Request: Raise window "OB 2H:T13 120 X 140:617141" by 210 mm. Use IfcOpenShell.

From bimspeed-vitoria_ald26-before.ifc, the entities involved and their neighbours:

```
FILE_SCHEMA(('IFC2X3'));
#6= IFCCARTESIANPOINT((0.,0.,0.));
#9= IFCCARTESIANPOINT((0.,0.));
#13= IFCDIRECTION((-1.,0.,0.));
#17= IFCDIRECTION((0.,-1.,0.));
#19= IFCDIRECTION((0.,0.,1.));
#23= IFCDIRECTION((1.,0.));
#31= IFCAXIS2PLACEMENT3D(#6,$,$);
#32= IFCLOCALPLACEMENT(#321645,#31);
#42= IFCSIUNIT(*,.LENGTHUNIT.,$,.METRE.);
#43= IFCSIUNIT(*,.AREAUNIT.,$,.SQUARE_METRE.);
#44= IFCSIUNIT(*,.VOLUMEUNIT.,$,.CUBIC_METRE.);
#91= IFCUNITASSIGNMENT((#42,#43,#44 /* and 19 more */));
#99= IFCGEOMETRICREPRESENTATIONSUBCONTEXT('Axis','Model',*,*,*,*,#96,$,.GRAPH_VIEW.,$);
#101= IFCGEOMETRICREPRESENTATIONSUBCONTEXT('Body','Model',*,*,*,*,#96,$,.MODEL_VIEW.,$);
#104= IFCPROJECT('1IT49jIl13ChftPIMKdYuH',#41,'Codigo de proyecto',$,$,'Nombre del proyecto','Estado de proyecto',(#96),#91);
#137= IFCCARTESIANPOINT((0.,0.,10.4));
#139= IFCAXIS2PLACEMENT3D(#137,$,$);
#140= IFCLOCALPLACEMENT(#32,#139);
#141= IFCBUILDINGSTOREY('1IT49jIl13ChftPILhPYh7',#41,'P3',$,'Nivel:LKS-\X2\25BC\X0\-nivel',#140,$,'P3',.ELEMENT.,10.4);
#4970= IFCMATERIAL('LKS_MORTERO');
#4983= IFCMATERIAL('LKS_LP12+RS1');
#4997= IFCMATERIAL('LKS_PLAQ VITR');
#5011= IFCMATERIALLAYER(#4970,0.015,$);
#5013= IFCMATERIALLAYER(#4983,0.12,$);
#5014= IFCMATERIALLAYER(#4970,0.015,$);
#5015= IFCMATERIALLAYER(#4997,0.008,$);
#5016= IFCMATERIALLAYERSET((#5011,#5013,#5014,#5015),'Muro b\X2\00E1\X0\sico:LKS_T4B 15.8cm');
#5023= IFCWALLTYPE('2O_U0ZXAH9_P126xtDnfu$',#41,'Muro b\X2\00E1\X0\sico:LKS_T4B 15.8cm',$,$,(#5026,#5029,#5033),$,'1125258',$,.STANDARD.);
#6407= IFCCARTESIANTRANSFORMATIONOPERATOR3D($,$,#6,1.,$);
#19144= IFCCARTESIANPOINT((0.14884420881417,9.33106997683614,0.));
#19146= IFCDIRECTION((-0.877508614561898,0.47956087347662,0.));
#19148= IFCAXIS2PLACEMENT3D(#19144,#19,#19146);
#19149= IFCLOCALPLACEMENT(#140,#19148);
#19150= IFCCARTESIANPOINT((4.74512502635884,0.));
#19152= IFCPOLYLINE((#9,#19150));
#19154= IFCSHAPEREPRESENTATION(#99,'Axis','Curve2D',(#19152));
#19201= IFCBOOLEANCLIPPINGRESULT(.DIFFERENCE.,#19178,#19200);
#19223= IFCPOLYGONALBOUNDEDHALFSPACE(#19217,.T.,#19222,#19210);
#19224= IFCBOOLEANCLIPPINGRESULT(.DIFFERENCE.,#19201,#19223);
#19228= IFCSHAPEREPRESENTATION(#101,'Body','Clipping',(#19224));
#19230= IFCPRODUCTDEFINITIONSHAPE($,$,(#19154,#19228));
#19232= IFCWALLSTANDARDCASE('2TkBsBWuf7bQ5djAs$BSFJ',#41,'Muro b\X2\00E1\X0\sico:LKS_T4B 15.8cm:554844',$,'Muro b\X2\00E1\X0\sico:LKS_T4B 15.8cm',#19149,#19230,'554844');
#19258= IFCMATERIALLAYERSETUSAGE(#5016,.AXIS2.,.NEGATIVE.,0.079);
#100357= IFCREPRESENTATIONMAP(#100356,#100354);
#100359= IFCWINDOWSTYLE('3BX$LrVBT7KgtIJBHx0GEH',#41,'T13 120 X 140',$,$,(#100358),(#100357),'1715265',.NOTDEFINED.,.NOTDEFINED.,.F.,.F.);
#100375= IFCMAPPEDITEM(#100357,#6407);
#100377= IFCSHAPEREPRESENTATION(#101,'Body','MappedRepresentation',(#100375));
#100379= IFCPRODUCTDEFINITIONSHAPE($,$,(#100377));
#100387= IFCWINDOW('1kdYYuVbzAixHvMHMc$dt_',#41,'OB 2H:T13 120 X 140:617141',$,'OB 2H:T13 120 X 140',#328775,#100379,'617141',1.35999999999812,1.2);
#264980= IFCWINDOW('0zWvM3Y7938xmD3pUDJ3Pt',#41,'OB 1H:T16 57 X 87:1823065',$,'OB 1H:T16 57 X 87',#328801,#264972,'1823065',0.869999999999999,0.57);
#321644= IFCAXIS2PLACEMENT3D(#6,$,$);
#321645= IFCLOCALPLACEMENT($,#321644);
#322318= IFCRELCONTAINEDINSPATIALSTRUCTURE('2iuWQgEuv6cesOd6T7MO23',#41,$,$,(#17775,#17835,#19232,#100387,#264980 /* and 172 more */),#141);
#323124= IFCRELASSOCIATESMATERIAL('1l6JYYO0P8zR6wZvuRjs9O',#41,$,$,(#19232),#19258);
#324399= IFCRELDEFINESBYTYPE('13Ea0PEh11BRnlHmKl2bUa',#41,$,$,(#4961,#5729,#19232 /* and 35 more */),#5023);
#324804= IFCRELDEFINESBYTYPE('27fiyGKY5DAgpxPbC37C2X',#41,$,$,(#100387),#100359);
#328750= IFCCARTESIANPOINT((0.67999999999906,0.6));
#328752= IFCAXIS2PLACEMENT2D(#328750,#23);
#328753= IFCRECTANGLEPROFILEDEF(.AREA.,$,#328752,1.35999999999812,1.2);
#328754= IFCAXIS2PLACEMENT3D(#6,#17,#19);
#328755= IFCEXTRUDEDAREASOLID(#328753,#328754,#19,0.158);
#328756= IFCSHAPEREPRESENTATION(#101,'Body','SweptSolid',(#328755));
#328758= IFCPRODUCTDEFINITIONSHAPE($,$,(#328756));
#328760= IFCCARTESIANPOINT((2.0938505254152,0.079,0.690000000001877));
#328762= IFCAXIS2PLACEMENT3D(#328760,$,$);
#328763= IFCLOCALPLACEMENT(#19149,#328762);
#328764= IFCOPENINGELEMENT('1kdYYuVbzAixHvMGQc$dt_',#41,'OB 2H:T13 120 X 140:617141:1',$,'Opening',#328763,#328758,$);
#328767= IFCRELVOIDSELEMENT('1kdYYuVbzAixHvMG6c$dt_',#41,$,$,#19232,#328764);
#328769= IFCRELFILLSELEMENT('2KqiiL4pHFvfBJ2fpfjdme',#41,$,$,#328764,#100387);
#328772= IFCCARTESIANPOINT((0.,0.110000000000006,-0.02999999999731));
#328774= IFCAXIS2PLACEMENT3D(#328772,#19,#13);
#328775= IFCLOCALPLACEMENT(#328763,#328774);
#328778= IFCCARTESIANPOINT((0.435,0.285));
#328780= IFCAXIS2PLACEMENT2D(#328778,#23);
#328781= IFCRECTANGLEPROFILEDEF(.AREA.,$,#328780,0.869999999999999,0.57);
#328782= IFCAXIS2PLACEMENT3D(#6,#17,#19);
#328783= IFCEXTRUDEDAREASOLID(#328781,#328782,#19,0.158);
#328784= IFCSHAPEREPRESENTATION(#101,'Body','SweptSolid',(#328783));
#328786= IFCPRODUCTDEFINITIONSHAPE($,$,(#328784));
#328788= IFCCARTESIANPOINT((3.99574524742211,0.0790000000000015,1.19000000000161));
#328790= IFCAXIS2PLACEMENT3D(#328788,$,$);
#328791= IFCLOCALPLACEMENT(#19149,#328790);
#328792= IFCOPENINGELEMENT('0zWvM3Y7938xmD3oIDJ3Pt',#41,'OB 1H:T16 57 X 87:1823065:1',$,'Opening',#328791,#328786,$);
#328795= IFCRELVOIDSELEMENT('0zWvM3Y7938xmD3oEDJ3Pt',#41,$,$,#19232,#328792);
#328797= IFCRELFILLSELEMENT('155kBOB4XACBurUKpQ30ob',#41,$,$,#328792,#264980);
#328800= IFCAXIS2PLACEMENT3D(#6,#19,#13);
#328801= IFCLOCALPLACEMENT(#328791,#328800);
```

```python
import numpy as np
import ifcopenshell
import ifcopenshell.api.geometry
import ifcopenshell.util.placement
import ifcopenshell.util.unit

model = ifcopenshell.open("bimspeed-vitoria_ald26-before.ifc")
unit_scale = ifcopenshell.util.unit.calculate_unit_scale(model)

window = model.by_guid("1kdYYuVbzAixHvMHMc$dt_")
opening = window.FillsVoids[0].RelatingOpeningElement
dz = 0.21 / unit_scale

shift = np.array([0.0, 0.0, dz])
# The window is placed relative to its opening, so it follows when the opening moves.
matrix = ifcopenshell.util.placement.get_local_placement(opening.ObjectPlacement)
matrix[:3, 3] += shift
ifcopenshell.api.geometry.edit_object_placement(
    model, product=opening, matrix=matrix, is_si=False, should_transform_children=True
)

print(f"moved by {dz * unit_scale:+.3f} m")

model.write("bimspeed-vitoria_ald26-before_v2.ifc")
```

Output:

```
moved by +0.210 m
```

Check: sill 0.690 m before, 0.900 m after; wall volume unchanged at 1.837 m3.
